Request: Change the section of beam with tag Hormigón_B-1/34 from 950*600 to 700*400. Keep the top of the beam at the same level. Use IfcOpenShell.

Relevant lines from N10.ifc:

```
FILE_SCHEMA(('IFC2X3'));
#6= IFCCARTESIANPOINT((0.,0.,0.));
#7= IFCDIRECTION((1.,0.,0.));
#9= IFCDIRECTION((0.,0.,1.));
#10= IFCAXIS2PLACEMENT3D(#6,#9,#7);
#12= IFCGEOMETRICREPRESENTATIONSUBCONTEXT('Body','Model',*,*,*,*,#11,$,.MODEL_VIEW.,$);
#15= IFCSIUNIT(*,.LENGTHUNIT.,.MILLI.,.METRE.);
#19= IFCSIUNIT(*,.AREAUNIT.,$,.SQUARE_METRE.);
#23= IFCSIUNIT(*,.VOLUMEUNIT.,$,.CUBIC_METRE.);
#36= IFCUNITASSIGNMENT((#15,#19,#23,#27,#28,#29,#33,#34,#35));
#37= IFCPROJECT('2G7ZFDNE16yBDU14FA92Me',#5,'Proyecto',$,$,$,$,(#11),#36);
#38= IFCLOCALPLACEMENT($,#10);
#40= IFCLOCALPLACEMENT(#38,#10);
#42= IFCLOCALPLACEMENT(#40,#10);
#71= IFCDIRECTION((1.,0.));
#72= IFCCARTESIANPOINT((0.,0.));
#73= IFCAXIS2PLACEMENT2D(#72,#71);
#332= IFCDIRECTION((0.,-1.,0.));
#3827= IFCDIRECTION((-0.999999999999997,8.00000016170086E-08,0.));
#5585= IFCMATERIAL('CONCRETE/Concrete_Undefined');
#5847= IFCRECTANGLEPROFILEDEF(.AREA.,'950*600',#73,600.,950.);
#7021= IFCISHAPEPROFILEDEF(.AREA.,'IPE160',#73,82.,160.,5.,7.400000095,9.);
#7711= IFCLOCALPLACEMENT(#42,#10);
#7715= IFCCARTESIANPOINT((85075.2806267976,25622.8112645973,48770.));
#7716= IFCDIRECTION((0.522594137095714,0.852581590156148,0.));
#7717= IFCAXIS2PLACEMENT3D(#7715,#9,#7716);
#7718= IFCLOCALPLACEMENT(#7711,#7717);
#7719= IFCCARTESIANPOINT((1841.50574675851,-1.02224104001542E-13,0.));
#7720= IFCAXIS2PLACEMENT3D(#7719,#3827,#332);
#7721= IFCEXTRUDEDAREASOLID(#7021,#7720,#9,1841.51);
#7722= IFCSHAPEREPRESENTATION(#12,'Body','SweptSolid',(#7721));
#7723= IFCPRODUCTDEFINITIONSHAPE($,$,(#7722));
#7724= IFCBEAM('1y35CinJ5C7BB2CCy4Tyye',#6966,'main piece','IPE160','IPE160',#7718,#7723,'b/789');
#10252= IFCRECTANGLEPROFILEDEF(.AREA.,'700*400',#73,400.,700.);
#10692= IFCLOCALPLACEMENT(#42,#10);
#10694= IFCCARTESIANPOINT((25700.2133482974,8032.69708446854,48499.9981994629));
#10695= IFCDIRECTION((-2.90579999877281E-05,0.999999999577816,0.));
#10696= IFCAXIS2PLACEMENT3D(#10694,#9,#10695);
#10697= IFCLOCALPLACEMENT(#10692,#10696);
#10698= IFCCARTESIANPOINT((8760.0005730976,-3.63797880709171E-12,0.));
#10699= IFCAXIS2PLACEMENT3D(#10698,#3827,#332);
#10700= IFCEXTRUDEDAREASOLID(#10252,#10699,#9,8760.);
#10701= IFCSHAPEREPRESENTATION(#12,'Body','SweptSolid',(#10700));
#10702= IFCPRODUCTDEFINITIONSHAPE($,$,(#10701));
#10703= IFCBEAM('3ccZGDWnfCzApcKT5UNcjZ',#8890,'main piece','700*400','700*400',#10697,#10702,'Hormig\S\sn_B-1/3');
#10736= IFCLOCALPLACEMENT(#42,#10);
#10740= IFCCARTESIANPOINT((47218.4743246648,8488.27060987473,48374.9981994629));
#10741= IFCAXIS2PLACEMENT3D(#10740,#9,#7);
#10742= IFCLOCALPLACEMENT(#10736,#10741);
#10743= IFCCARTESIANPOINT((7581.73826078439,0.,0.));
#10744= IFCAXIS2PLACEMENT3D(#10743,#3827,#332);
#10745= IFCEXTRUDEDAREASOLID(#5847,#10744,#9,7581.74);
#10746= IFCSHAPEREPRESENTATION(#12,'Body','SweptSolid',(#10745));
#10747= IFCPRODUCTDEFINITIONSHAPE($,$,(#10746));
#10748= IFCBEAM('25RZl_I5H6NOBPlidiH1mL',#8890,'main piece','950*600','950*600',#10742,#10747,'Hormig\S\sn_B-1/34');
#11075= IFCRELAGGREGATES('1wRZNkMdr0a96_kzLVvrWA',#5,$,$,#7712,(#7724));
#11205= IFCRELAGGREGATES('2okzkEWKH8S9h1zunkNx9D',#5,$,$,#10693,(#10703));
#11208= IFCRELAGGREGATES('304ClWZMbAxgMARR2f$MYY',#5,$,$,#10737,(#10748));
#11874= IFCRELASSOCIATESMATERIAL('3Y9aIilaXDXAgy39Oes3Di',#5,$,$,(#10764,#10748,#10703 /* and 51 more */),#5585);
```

```python
import ifcopenshell
import ifcopenshell.util.element
import ifcopenshell.util.representation

model = ifcopenshell.open("N10.ifc")

member = model.by_guid("25RZl_I5H6NOBPlidiH1mL")
source = next(p for p in model.by_type("IfcRectangleProfileDef") if p.ProfileName == "700*400")

body = ifcopenshell.util.representation.get_representation(member, "Model", "Body")
solid = body.Items[0]
old_profile = solid.SweptArea

# Copy the section's sizes but keep this member's own profile position.
profile = ifcopenshell.util.element.copy(model, source)
# Profiles are centred, so shift by half the change in depth to hold the top.
shift = (old_profile.YDim - profile.YDim) / 2
x, y = old_profile.Position.Location.Coordinates
up = (0.0, 1.0)  # upwards, in the solid's own plane
location = model.createIfcCartesianPoint((x + up[0] * shift, y + up[1] * shift))
profile.Position = model.createIfcAxis2Placement2D(location, old_profile.Position.RefDirection)
solid.SweptArea = profile
if not model.get_total_inverses(old_profile):
    ifcopenshell.util.element.remove_deep2(model, old_profile)
member.Description = member.Description.replace("950*600", "700*400")
member.ObjectType = member.ObjectType.replace("950*600", "700*400")

print(solid.SweptArea)

model.write("N10_v2.ifc")
```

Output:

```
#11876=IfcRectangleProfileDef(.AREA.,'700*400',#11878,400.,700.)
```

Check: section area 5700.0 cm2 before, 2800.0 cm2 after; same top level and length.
